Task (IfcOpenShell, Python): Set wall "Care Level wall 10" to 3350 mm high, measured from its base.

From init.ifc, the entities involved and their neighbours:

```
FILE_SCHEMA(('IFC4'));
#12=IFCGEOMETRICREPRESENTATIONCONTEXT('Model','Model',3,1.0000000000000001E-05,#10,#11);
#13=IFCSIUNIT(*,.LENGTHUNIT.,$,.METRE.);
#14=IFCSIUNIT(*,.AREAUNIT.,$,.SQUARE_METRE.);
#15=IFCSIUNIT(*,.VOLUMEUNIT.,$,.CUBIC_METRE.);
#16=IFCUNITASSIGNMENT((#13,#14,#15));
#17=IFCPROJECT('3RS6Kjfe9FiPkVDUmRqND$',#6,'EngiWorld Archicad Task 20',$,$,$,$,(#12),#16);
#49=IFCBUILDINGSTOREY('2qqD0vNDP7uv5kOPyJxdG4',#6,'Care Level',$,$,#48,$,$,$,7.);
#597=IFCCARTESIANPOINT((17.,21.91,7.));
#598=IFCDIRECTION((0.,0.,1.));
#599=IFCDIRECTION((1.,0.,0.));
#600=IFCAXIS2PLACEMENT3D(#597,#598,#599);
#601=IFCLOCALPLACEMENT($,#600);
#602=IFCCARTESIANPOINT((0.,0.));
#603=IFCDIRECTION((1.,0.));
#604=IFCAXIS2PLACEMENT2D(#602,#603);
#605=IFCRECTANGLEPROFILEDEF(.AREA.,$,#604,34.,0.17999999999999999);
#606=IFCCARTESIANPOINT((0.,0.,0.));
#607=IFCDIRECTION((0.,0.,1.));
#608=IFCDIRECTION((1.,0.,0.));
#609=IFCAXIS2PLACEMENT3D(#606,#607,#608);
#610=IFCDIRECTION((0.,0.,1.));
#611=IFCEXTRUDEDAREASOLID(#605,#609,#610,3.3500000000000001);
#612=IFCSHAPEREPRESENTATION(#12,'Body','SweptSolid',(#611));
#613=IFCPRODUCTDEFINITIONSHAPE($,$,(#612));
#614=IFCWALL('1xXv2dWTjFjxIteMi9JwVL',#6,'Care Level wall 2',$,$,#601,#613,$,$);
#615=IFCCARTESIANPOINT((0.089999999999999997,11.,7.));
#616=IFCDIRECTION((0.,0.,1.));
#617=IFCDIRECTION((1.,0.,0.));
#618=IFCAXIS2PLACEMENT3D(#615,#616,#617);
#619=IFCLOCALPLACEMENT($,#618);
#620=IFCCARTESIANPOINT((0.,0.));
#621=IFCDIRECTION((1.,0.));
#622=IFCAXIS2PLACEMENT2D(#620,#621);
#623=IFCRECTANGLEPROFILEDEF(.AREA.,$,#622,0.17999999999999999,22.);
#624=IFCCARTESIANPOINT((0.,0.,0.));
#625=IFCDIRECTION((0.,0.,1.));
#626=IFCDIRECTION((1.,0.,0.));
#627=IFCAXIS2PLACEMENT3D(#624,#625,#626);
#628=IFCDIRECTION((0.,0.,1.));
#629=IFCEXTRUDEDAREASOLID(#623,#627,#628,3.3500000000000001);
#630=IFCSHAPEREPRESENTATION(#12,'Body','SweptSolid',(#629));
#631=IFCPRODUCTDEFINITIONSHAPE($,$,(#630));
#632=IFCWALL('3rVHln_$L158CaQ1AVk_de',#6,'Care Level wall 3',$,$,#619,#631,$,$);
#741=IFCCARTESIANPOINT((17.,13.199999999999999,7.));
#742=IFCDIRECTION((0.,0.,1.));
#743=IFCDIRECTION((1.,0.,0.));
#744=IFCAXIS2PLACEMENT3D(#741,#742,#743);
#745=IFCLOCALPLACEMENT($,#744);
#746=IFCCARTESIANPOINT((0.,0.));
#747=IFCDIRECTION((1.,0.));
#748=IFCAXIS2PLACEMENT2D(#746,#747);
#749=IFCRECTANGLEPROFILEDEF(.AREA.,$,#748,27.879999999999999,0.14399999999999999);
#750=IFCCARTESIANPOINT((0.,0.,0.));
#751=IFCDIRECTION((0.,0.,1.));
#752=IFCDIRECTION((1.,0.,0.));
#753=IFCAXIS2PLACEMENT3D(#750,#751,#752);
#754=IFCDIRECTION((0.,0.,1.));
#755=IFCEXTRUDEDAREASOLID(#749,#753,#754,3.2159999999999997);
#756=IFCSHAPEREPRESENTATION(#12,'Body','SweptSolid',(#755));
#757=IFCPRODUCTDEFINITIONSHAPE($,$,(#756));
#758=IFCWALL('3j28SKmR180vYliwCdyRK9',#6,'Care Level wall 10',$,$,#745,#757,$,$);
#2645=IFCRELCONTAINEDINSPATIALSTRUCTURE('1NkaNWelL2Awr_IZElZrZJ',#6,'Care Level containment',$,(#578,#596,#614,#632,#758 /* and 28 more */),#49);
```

```python
import ifcopenshell
import ifcopenshell.geom
import ifcopenshell.util.shape
import ifcopenshell.util.unit

model = ifcopenshell.open("init.ifc")
unit_scale = ifcopenshell.util.unit.calculate_unit_scale(model)
settings = ifcopenshell.geom.settings()


def volume(element):
    """Net volume in cubic metres, openings subtracted."""
    shape = ifcopenshell.geom.create_shape(settings, element)
    return ifcopenshell.util.shape.get_volume(shape.geometry)


wall = model.by_id(758)
before = volume(wall)

body = next(r for r in wall.Representation.Representations if r.RepresentationIdentifier == "Body")
solid = body.Items[0]
old_height = solid.Depth
solid.Depth = 3.35 / unit_scale
after = volume(wall)

print(f"height {old_height:g} -> {solid.Depth:g}, volume {before:.3f} -> {after:.3f} m3")

model.write("init_rev.ifc")
```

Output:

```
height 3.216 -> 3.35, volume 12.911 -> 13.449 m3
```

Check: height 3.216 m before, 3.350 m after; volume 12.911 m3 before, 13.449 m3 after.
